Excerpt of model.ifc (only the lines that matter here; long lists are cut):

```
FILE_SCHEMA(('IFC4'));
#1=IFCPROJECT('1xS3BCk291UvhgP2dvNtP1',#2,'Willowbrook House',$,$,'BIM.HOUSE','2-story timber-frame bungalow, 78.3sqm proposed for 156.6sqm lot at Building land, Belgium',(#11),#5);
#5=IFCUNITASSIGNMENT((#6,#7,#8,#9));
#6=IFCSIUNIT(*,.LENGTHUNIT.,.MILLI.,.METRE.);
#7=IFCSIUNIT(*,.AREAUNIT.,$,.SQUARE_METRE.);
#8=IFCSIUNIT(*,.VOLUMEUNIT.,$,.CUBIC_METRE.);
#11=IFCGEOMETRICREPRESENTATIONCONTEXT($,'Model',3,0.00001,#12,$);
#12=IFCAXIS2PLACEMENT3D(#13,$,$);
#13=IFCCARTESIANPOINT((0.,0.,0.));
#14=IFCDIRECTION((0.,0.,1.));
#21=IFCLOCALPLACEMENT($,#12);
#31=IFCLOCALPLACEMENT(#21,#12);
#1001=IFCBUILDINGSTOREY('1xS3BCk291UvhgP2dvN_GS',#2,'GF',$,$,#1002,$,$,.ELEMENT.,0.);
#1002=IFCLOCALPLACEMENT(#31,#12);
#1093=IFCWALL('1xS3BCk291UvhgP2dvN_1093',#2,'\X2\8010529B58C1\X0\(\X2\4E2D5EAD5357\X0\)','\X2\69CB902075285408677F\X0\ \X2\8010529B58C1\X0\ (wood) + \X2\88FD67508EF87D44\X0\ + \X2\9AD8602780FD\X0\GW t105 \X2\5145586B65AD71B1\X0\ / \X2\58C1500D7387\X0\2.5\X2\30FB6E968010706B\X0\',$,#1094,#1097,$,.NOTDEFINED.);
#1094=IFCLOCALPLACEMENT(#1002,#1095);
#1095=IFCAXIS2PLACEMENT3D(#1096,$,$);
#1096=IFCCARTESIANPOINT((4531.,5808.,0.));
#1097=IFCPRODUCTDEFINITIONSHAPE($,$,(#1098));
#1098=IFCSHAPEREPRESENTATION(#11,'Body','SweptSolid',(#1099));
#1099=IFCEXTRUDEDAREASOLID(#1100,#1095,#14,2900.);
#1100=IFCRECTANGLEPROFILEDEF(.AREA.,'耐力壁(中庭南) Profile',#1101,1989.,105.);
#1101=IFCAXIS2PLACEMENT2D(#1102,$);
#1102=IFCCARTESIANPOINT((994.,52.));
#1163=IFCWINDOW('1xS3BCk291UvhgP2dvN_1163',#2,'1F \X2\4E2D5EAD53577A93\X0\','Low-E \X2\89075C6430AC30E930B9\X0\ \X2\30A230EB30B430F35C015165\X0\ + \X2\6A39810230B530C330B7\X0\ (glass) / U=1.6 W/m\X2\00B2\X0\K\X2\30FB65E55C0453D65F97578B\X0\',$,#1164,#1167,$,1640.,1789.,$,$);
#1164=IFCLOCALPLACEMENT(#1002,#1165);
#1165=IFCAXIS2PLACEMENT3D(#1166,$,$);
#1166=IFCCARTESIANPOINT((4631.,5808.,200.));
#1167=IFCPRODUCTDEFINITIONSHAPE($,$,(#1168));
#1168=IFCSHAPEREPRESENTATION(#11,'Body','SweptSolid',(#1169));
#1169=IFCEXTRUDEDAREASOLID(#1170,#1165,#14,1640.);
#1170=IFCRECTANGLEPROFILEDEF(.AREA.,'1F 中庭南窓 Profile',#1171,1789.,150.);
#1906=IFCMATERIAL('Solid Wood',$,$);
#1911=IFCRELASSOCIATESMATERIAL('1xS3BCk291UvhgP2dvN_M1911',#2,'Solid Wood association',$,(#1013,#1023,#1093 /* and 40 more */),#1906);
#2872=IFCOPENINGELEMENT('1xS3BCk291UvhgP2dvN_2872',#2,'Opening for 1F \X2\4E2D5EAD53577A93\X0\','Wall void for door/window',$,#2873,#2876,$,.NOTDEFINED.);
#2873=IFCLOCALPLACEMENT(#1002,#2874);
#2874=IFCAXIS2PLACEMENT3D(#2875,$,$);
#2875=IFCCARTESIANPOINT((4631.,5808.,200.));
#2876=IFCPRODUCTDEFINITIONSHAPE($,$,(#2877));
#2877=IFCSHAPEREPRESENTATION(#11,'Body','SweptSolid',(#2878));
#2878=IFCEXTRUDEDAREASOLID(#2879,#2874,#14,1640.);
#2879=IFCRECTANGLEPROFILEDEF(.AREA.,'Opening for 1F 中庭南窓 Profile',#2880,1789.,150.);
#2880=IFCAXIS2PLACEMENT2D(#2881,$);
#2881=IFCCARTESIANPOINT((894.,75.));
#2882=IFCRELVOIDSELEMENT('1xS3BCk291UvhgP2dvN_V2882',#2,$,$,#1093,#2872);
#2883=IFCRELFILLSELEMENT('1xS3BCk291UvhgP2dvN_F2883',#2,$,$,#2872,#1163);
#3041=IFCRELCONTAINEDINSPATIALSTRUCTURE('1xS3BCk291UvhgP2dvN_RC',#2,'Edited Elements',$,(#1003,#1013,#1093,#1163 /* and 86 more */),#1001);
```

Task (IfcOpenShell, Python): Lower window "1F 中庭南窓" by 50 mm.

```python
import numpy as np
import ifcopenshell
import ifcopenshell.api.geometry
import ifcopenshell.util.placement
import ifcopenshell.util.unit

model = ifcopenshell.open("model.ifc")
unit_scale = ifcopenshell.util.unit.calculate_unit_scale(model)

window = model.by_guid("1xS3BCk291UvhgP2dvN_1163")
opening = window.FillsVoids[0].RelatingOpeningElement
dz = -0.05 / unit_scale

shift = np.array([0.0, 0.0, dz])
# The window is not placed relative to its opening, so move both.
for product in (opening, window):
    matrix = ifcopenshell.util.placement.get_local_placement(product.ObjectPlacement)
    matrix[:3, 3] += shift
    ifcopenshell.api.geometry.edit_object_placement(model, product=product, matrix=matrix, is_si=False)

print(f"moved by {dz * unit_scale:+.3f} m")

model.write("model_rev.ifc")
```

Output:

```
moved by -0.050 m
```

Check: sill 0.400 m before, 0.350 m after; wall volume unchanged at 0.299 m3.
